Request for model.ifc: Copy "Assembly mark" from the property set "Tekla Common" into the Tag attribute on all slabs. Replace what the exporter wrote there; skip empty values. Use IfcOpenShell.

First a look at what the model holds.

```python
import ifcopenshell
import ifcopenshell.util.element

model = ifcopenshell.open("model.ifc")
print(model.schema)
slabs = model.by_type("IfcSlab")
print(len(slabs), "slabs")
for e in slabs[:8]:
    source = ifcopenshell.util.element.get_pset(e, "Tekla Common", "Assembly mark")
    target = e.Tag
    print(e.id(), repr(source), repr(target), sep=" | ")
```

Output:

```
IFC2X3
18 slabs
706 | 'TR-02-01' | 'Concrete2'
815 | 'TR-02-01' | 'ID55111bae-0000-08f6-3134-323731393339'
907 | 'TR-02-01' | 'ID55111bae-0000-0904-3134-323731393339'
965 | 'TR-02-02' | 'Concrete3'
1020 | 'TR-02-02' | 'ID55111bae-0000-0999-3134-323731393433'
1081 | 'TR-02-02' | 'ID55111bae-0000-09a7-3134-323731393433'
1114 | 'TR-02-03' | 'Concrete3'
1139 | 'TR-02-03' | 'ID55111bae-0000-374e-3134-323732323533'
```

```python
import ifcopenshell
import ifcopenshell.util.element

model = ifcopenshell.open("model.ifc")

count = 0
for e in model.by_type("IfcSlab"):
    value = ifcopenshell.util.element.get_pset(e, "Tekla Common", "Assembly mark")
    current = e.Tag
    if not value or not value.strip() or current == value:
        continue
    e.Tag = value
    count += 1

print(count, "slabs updated")

model.write("model_updated.ifc")
```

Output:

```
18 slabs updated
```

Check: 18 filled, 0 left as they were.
